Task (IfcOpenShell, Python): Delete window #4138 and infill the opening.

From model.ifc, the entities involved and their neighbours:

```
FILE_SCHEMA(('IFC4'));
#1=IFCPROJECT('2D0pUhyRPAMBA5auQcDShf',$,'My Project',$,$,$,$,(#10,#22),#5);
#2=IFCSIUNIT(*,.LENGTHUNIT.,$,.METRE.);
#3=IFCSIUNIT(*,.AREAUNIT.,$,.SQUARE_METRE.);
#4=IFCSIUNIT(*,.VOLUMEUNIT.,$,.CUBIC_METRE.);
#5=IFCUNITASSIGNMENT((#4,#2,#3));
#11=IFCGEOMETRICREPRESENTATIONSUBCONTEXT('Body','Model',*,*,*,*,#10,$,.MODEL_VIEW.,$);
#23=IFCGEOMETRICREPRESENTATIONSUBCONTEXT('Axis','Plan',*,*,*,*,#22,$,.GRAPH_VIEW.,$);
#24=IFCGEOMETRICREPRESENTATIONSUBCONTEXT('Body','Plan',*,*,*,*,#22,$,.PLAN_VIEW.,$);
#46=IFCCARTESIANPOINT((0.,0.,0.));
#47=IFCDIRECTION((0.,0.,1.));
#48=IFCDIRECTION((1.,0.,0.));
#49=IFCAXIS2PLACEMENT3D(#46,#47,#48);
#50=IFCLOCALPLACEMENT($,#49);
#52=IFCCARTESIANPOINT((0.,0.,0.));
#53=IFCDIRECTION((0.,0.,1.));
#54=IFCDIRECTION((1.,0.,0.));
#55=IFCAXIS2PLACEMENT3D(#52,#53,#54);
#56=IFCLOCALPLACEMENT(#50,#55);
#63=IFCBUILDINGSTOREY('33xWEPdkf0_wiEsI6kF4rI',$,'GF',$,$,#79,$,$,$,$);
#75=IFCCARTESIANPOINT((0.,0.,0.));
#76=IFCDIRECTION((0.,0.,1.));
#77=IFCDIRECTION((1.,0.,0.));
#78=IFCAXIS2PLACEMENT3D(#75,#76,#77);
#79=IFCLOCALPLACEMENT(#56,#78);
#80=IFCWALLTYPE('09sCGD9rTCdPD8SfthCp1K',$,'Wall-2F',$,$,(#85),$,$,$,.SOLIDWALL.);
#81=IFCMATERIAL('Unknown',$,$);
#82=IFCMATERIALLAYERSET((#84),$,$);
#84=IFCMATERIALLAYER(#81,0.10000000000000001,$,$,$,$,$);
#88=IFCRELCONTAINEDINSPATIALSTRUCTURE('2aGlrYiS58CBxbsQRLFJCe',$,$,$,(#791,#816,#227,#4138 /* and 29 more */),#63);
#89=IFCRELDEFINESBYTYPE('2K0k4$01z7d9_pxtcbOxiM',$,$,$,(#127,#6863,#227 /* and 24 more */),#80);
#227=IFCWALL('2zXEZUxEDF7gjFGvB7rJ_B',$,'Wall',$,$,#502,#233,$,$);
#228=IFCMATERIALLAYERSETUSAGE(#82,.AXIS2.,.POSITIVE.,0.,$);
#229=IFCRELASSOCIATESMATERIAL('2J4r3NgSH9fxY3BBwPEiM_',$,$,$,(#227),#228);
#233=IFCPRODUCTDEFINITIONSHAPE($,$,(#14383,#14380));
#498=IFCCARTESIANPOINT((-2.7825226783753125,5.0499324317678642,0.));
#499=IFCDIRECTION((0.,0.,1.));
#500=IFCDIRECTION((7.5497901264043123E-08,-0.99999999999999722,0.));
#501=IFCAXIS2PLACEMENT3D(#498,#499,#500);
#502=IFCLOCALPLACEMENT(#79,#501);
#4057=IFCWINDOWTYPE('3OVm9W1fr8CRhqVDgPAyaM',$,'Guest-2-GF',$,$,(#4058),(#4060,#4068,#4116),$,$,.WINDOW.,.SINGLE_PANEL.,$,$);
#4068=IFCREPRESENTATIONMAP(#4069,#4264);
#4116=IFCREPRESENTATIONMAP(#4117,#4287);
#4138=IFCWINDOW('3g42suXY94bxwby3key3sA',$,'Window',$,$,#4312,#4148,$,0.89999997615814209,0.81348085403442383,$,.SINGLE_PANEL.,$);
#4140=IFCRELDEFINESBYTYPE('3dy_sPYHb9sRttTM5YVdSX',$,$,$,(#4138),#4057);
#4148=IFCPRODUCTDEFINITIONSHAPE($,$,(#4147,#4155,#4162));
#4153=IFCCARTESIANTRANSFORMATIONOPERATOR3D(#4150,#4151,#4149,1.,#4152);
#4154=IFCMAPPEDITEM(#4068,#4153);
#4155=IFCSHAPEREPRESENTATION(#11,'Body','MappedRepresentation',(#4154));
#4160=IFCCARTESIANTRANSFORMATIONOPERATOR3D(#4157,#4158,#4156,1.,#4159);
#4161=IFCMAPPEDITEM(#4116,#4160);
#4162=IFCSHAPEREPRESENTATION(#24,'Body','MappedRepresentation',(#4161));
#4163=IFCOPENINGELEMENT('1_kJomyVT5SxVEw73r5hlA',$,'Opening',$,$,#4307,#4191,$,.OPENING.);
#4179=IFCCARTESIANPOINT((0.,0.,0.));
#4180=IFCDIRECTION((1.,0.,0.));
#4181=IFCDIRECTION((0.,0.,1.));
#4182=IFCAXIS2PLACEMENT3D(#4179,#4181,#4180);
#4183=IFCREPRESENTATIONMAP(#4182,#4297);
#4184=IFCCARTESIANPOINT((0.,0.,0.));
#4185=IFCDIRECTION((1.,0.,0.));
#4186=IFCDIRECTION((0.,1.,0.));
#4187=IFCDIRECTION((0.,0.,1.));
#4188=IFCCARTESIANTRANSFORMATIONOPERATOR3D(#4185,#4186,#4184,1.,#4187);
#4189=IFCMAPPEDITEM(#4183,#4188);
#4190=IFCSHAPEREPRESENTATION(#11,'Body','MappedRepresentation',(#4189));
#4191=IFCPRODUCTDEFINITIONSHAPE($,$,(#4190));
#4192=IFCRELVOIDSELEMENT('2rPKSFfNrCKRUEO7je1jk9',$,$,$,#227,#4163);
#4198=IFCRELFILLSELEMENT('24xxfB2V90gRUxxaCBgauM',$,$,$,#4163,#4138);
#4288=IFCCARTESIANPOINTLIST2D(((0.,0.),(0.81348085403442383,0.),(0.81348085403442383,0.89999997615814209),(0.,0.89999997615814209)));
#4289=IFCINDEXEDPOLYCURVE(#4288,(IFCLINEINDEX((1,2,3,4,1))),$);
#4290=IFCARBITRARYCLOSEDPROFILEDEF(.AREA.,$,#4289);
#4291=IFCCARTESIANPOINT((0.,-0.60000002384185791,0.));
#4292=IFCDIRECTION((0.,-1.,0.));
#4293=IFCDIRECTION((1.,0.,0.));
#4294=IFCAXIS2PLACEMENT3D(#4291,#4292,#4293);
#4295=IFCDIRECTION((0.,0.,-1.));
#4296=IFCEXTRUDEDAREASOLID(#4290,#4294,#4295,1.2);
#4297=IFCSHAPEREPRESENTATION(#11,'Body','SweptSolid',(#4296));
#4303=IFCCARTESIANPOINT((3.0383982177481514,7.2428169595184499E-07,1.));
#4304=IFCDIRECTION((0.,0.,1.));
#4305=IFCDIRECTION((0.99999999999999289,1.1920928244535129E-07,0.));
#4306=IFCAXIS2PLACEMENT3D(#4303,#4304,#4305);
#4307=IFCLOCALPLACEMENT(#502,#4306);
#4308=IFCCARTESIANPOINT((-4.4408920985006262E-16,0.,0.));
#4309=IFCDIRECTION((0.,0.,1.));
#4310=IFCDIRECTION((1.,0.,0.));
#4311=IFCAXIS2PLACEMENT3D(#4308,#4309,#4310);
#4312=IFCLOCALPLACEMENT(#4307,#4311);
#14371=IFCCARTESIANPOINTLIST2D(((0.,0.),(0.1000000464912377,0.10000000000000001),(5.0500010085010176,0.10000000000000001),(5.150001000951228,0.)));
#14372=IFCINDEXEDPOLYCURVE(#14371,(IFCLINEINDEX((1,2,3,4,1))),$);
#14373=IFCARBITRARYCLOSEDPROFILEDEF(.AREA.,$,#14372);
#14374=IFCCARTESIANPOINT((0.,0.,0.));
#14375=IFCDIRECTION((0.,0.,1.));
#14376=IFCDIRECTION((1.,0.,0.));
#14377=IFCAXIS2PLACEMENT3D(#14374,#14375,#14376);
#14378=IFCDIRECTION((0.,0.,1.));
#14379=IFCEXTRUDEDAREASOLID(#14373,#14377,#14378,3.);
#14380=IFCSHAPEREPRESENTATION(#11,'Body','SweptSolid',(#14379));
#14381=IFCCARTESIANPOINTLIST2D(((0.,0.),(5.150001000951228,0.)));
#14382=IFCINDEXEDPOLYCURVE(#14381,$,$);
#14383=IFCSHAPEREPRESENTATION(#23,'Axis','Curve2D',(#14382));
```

```python
import ifcopenshell
import ifcopenshell.api.feature
import ifcopenshell.api.root
import ifcopenshell.geom
import ifcopenshell.util.shape

model = ifcopenshell.open("model.ifc")
settings = ifcopenshell.geom.settings()


def volume(element):
    """Net volume in cubic metres, openings subtracted."""
    shape = ifcopenshell.geom.create_shape(settings, element)
    return ifcopenshell.util.shape.get_volume(shape.geometry)


window = model.by_id(4138)
opening = window.FillsVoids[0].RelatingOpeningElement
wall = opening.VoidsElements[0].RelatingBuildingElement
before = volume(wall)

ifcopenshell.api.root.remove_product(model, product=window)
ifcopenshell.api.feature.remove_feature(model, feature=opening)

after = volume(wall)

print(f"wall volume {before:.3f} -> {after:.3f} m3")

model.write("model_edited.ifc")
```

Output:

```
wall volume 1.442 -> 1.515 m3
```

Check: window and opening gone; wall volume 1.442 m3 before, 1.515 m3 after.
